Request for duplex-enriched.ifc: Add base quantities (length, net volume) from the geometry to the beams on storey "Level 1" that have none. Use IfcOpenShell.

First a look at what the model holds.

```python
import ifcopenshell
import ifcopenshell.util.element
import ifcopenshell.util.unit

model = ifcopenshell.open("duplex-enriched.ifc")
print(model.schema)
for unit_type in ("LENGTHUNIT", "AREAUNIT", "VOLUMEUNIT"):
    print(unit_type, ifcopenshell.util.unit.calculate_unit_scale(model, unit_type))
storey = next(s for s in model.by_type("IfcBuildingStorey") if s.Name == "Level 1")
beams = [e for e in ifcopenshell.util.element.get_decomposition(storey) if e.is_a("IfcBeam")]
for e in sorted(beams, key=lambda e: e.id()):
    print(e.id(), e.is_a(), e.Name, list(ifcopenshell.util.element.get_psets(e, qtos_only=True)), sep=" | ")
```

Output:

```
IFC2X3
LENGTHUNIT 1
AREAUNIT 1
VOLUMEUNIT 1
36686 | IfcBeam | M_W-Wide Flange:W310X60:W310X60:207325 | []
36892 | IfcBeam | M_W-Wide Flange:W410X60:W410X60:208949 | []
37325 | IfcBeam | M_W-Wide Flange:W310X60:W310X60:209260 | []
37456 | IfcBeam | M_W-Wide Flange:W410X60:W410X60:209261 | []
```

```python
import ifcopenshell
import ifcopenshell.api.pset
import ifcopenshell.geom
import ifcopenshell.util.element
import ifcopenshell.util.shape
import ifcopenshell.util.unit

model = ifcopenshell.open("duplex-enriched.ifc")
unit_scale = ifcopenshell.util.unit.calculate_unit_scale(model)
volume_scale = ifcopenshell.util.unit.calculate_unit_scale(model, "VOLUMEUNIT")
settings = ifcopenshell.geom.settings()

storey = next(s for s in model.by_type("IfcBuildingStorey") if s.Name == "Level 1")
beams = [e for e in ifcopenshell.util.element.get_decomposition(storey) if e.is_a("IfcBeam")]

for e in sorted(beams, key=lambda e: e.id()):
    if ifcopenshell.util.element.get_psets(e, qtos_only=True, should_inherit=False):
        continue
    # Geometry comes back in metres, in the element's own axes.
    shape = ifcopenshell.geom.create_shape(settings, e)
    values = {
        "Length": ifcopenshell.util.shape.get_max_xyz(shape.geometry) / unit_scale,
        "NetVolume": ifcopenshell.util.shape.get_volume(shape.geometry) / volume_scale,
    }
    qto = ifcopenshell.api.pset.add_qto(model, product=e, name="BaseQuantities")
    ifcopenshell.api.pset.edit_qto(model, qto=qto, properties=values)
    print(e.id(), {k: round(v, 3) for k, v in values.items()})

model.write("duplex-enriched_updated.ifc")
```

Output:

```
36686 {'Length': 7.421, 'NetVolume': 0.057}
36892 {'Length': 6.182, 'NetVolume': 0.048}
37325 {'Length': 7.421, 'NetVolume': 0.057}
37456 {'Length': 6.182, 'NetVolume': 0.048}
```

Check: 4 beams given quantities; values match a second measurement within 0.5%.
